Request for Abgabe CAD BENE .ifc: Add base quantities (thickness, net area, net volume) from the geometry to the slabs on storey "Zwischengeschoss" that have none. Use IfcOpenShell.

First a look at what the model holds.

```python
import ifcopenshell
import ifcopenshell.util.element
import ifcopenshell.util.unit

model = ifcopenshell.open("Abgabe CAD BENE .ifc")
print(model.schema)
for unit_type in ("LENGTHUNIT", "AREAUNIT", "VOLUMEUNIT"):
    print(unit_type, ifcopenshell.util.unit.calculate_unit_scale(model, unit_type))
storey = next(s for s in model.by_type("IfcBuildingStorey") if s.Name == "Zwischengeschoss")
slabs = [e for e in ifcopenshell.util.element.get_decomposition(storey) if e.is_a("IfcSlab")]
for e in sorted(slabs, key=lambda e: e.id()):
    print(e.id(), e.is_a(), e.Name, list(ifcopenshell.util.element.get_psets(e, qtos_only=True)), sep=" | ")
```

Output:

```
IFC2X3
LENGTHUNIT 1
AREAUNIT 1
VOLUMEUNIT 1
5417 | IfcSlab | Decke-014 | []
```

```python
import ifcopenshell
import ifcopenshell.api.pset
import ifcopenshell.geom
import ifcopenshell.util.element
import ifcopenshell.util.shape
import ifcopenshell.util.unit

model = ifcopenshell.open("Abgabe CAD BENE .ifc")
unit_scale = ifcopenshell.util.unit.calculate_unit_scale(model)
area_scale = ifcopenshell.util.unit.calculate_unit_scale(model, "AREAUNIT")
volume_scale = ifcopenshell.util.unit.calculate_unit_scale(model, "VOLUMEUNIT")
settings = ifcopenshell.geom.settings()

storey = next(s for s in model.by_type("IfcBuildingStorey") if s.Name == "Zwischengeschoss")
slabs = [e for e in ifcopenshell.util.element.get_decomposition(storey) if e.is_a("IfcSlab")]

for e in sorted(slabs, key=lambda e: e.id()):
    if ifcopenshell.util.element.get_psets(e, qtos_only=True, should_inherit=False):
        continue
    # Geometry comes back in metres, in the element's own axes.
    shape = ifcopenshell.geom.create_shape(settings, e)
    values = {
        "Width": ifcopenshell.util.shape.get_z(shape.geometry) / unit_scale,
        "NetArea": ifcopenshell.util.shape.get_footprint_area(shape.geometry) / area_scale,
        "NetVolume": ifcopenshell.util.shape.get_volume(shape.geometry) / volume_scale,
    }
    qto = ifcopenshell.api.pset.add_qto(model, product=e, name="BaseQuantities")
    ifcopenshell.api.pset.edit_qto(model, qto=qto, properties=values)
    print(e.id(), {k: round(v, 3) for k, v in values.items()})

model.write("Abgabe CAD BENE -out.ifc")
```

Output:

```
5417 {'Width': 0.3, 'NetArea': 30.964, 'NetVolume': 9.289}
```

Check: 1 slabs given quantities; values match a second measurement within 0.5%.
